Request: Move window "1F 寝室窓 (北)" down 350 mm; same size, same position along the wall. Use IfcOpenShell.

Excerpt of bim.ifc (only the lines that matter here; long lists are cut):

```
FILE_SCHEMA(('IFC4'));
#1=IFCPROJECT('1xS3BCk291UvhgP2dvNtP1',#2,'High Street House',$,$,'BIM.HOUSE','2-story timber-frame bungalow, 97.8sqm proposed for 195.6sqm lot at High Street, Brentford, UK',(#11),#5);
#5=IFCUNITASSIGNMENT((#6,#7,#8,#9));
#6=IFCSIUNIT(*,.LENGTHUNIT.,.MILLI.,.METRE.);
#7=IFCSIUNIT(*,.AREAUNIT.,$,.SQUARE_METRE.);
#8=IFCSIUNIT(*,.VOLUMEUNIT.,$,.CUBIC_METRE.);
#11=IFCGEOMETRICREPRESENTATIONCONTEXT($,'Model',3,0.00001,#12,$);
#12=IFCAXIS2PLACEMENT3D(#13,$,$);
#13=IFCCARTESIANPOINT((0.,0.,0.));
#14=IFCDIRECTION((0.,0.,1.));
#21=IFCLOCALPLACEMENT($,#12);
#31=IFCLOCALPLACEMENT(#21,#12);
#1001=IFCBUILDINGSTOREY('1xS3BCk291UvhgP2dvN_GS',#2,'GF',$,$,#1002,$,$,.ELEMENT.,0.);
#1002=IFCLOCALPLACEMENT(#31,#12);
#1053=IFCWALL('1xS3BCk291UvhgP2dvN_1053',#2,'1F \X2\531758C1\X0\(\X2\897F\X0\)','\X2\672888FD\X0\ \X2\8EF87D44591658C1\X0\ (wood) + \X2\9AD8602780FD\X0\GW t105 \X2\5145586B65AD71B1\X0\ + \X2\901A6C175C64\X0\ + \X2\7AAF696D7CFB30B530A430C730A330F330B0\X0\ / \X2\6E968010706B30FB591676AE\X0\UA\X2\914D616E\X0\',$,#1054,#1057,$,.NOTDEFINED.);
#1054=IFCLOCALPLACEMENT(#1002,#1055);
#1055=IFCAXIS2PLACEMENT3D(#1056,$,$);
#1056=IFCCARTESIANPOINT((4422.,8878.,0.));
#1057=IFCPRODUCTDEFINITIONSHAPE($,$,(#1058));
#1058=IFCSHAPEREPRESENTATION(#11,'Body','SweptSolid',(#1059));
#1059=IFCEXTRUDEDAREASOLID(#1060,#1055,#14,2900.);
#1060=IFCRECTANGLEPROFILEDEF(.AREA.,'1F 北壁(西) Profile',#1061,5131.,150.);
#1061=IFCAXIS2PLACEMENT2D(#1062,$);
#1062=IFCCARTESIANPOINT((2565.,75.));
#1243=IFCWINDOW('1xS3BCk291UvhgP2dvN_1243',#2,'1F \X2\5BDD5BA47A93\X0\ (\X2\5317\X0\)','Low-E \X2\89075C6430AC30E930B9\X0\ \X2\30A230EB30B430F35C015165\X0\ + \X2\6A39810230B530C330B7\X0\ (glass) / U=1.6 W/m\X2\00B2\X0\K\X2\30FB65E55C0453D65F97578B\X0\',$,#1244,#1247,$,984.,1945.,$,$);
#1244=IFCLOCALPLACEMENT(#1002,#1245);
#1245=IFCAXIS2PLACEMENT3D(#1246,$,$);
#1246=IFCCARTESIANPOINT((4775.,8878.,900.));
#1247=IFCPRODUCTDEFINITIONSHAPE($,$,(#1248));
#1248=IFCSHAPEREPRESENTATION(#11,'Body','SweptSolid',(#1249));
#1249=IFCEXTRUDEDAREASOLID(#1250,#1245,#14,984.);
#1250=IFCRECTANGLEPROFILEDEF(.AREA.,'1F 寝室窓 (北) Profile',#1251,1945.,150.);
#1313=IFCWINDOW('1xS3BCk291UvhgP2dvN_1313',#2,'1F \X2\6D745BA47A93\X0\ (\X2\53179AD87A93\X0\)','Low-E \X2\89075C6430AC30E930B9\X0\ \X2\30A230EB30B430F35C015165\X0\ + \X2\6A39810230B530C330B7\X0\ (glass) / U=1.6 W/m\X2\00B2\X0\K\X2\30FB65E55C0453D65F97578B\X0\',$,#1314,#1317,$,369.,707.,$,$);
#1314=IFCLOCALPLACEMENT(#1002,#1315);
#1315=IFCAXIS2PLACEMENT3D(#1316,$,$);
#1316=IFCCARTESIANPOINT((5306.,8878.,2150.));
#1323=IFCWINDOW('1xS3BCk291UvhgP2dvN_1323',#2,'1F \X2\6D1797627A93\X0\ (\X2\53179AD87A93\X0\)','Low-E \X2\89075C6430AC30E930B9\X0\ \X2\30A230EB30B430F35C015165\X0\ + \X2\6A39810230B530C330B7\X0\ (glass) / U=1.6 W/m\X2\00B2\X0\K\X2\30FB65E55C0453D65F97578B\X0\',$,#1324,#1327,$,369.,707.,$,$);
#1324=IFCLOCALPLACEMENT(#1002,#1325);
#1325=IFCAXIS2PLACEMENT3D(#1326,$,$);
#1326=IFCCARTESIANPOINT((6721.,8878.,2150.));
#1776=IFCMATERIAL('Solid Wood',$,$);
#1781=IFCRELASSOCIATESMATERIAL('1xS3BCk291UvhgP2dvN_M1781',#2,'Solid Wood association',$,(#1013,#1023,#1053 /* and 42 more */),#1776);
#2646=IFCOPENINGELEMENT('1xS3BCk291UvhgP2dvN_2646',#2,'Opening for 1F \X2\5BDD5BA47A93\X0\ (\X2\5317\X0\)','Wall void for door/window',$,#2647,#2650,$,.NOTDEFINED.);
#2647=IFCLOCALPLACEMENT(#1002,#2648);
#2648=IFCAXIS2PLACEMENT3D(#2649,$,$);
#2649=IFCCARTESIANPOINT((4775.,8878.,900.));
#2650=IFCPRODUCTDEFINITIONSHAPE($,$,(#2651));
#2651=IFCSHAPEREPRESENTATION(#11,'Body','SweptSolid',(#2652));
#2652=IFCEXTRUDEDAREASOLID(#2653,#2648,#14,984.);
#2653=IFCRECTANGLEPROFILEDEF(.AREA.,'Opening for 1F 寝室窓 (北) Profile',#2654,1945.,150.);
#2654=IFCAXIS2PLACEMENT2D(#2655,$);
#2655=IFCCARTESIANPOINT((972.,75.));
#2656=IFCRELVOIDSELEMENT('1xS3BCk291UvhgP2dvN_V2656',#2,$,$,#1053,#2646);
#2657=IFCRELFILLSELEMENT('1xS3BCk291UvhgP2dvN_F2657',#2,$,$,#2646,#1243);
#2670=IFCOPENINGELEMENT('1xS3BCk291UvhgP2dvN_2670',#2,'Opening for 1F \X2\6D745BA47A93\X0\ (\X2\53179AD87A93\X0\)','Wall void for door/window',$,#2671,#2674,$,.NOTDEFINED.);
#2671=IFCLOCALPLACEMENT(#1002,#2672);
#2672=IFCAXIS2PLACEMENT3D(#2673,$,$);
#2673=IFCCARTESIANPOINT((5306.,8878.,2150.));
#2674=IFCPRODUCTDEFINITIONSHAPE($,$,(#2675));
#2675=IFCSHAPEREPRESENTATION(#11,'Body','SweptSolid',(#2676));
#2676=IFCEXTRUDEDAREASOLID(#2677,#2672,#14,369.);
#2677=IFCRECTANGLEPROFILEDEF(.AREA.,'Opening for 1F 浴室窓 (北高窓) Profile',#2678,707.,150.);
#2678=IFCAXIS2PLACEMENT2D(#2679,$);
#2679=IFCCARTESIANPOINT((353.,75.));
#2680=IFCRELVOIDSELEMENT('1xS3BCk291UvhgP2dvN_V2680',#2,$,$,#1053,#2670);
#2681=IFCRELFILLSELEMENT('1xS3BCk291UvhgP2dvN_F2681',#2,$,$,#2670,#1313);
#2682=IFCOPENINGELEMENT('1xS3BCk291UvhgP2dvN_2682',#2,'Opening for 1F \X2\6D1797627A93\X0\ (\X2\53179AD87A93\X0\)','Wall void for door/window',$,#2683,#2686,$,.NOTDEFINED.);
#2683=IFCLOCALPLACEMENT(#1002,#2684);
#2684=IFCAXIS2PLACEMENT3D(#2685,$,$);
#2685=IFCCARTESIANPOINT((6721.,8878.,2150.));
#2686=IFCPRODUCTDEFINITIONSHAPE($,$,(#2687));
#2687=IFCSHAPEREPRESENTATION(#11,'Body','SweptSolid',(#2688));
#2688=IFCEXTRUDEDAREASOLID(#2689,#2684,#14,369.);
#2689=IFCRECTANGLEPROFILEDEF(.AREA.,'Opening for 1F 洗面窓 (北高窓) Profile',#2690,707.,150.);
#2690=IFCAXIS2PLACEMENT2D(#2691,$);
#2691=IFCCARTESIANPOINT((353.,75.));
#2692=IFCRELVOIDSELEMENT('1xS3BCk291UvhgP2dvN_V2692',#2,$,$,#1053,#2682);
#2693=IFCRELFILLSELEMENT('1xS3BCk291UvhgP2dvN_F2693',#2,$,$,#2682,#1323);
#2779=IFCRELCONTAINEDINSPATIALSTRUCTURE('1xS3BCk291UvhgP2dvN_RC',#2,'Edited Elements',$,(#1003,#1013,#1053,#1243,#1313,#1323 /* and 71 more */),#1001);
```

```python
import numpy as np
import ifcopenshell
import ifcopenshell.api.geometry
import ifcopenshell.util.placement
import ifcopenshell.util.unit

model = ifcopenshell.open("bim.ifc")
unit_scale = ifcopenshell.util.unit.calculate_unit_scale(model)

window = model.by_id(1243)
opening = window.FillsVoids[0].RelatingOpeningElement
dz = -350.0

shift = np.array([0.0, 0.0, dz])
# The window is not placed relative to its opening, so move both.
for product in (opening, window):
    matrix = ifcopenshell.util.placement.get_local_placement(product.ObjectPlacement)
    matrix[:3, 3] += shift
    ifcopenshell.api.geometry.edit_object_placement(model, product=product, matrix=matrix, is_si=False)

print(f"moved by {dz * unit_scale:+.3f} m")

model.write("bim-out.ifc")
```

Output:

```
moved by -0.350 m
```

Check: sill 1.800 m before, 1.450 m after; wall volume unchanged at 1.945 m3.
